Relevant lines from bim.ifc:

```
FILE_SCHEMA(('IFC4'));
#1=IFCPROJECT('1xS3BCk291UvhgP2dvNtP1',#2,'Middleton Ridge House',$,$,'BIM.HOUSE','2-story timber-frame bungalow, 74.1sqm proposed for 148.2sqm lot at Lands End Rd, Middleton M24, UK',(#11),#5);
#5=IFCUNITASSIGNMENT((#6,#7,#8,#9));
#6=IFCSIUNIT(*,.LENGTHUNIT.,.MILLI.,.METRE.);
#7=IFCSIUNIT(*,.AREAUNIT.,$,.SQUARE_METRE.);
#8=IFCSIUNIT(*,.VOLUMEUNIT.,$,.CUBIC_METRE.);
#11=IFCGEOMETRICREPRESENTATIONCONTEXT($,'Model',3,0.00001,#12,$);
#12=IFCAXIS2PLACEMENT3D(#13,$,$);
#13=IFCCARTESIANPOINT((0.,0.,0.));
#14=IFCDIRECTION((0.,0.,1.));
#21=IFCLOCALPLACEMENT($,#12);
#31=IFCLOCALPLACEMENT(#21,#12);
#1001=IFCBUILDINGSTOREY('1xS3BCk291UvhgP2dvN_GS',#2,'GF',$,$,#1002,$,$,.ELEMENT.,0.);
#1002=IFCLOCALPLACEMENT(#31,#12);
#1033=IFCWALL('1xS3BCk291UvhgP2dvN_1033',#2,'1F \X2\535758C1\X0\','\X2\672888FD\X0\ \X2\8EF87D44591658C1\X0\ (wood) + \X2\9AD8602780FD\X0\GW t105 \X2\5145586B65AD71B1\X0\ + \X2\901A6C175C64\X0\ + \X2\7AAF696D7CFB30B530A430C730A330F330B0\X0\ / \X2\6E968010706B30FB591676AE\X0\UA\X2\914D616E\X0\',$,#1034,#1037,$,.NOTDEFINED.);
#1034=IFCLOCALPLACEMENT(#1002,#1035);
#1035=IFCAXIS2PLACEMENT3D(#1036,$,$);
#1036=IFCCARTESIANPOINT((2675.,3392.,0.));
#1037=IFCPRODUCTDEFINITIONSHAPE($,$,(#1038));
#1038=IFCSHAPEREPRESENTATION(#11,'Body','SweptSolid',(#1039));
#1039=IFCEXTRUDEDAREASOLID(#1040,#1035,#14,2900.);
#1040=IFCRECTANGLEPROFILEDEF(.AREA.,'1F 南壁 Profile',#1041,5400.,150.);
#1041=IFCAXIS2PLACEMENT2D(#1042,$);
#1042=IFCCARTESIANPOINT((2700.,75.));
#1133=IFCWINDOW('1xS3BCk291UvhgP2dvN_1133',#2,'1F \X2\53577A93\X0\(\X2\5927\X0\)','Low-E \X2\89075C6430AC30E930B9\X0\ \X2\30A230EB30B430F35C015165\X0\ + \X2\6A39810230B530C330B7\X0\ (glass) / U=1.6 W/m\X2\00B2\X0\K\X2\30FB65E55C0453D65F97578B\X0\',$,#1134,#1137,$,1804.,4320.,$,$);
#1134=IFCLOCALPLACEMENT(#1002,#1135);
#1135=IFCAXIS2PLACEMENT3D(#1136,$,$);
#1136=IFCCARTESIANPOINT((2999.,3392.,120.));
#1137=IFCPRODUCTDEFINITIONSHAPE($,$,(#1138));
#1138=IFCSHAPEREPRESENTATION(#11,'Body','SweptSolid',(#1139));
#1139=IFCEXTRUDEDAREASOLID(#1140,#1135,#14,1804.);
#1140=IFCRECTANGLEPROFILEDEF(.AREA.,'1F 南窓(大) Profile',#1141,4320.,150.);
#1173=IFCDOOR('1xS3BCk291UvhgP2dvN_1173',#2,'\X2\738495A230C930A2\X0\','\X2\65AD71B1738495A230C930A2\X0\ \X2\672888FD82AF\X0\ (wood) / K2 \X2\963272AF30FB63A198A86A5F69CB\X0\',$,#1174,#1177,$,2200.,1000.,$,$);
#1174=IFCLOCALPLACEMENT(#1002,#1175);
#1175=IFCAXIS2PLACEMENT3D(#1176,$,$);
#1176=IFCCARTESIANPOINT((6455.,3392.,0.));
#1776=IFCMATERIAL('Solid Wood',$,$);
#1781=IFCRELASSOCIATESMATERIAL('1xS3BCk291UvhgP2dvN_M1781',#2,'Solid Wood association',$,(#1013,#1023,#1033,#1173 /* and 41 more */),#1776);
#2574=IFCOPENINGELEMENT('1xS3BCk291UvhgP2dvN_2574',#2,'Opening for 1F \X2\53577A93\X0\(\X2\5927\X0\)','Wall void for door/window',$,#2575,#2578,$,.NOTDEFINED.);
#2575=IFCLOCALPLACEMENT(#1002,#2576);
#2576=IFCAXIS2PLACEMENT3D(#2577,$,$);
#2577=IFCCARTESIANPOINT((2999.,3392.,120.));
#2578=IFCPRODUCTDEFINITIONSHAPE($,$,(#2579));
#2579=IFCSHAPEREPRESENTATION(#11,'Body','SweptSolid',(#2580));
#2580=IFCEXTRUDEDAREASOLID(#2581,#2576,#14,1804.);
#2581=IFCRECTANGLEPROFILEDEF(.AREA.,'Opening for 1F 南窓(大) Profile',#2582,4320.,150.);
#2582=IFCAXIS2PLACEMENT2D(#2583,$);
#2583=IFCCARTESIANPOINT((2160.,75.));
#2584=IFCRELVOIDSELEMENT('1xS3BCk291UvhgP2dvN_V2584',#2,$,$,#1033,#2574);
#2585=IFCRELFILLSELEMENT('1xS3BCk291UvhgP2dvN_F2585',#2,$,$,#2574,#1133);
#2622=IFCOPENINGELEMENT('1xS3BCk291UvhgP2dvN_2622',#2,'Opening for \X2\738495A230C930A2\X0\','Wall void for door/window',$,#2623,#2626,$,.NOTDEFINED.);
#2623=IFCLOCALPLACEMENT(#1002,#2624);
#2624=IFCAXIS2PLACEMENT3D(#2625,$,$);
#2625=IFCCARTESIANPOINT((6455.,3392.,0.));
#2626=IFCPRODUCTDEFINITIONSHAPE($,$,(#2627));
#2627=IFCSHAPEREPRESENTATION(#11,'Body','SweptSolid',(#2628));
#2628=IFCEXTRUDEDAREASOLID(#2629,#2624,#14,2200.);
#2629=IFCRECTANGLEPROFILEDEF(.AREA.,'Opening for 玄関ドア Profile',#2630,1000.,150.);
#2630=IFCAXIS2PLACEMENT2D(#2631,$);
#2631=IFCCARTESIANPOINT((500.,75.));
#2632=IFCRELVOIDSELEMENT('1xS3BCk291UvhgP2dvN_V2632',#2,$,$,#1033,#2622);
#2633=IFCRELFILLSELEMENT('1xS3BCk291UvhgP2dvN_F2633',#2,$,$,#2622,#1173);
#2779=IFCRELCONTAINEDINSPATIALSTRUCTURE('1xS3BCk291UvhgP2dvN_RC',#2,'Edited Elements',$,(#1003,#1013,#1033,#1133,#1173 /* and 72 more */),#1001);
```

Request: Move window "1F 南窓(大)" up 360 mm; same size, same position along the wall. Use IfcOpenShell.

```python
import numpy as np
import ifcopenshell
import ifcopenshell.api.geometry
import ifcopenshell.util.placement
import ifcopenshell.util.unit

model = ifcopenshell.open("bim.ifc")
unit_scale = ifcopenshell.util.unit.calculate_unit_scale(model)

window = model.by_id(1133)
opening = window.FillsVoids[0].RelatingOpeningElement
dz = 360.0

shift = np.array([0.0, 0.0, dz])
# The window is not placed relative to its opening, so move both.
for product in (opening, window):
    matrix = ifcopenshell.util.placement.get_local_placement(product.ObjectPlacement)
    matrix[:3, 3] += shift
    ifcopenshell.api.geometry.edit_object_placement(model, product=product, matrix=matrix, is_si=False)

print(f"moved by {dz * unit_scale:+.3f} m")

model.write("bim_rev.ifc")
```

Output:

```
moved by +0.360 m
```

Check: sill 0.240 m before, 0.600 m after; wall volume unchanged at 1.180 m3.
